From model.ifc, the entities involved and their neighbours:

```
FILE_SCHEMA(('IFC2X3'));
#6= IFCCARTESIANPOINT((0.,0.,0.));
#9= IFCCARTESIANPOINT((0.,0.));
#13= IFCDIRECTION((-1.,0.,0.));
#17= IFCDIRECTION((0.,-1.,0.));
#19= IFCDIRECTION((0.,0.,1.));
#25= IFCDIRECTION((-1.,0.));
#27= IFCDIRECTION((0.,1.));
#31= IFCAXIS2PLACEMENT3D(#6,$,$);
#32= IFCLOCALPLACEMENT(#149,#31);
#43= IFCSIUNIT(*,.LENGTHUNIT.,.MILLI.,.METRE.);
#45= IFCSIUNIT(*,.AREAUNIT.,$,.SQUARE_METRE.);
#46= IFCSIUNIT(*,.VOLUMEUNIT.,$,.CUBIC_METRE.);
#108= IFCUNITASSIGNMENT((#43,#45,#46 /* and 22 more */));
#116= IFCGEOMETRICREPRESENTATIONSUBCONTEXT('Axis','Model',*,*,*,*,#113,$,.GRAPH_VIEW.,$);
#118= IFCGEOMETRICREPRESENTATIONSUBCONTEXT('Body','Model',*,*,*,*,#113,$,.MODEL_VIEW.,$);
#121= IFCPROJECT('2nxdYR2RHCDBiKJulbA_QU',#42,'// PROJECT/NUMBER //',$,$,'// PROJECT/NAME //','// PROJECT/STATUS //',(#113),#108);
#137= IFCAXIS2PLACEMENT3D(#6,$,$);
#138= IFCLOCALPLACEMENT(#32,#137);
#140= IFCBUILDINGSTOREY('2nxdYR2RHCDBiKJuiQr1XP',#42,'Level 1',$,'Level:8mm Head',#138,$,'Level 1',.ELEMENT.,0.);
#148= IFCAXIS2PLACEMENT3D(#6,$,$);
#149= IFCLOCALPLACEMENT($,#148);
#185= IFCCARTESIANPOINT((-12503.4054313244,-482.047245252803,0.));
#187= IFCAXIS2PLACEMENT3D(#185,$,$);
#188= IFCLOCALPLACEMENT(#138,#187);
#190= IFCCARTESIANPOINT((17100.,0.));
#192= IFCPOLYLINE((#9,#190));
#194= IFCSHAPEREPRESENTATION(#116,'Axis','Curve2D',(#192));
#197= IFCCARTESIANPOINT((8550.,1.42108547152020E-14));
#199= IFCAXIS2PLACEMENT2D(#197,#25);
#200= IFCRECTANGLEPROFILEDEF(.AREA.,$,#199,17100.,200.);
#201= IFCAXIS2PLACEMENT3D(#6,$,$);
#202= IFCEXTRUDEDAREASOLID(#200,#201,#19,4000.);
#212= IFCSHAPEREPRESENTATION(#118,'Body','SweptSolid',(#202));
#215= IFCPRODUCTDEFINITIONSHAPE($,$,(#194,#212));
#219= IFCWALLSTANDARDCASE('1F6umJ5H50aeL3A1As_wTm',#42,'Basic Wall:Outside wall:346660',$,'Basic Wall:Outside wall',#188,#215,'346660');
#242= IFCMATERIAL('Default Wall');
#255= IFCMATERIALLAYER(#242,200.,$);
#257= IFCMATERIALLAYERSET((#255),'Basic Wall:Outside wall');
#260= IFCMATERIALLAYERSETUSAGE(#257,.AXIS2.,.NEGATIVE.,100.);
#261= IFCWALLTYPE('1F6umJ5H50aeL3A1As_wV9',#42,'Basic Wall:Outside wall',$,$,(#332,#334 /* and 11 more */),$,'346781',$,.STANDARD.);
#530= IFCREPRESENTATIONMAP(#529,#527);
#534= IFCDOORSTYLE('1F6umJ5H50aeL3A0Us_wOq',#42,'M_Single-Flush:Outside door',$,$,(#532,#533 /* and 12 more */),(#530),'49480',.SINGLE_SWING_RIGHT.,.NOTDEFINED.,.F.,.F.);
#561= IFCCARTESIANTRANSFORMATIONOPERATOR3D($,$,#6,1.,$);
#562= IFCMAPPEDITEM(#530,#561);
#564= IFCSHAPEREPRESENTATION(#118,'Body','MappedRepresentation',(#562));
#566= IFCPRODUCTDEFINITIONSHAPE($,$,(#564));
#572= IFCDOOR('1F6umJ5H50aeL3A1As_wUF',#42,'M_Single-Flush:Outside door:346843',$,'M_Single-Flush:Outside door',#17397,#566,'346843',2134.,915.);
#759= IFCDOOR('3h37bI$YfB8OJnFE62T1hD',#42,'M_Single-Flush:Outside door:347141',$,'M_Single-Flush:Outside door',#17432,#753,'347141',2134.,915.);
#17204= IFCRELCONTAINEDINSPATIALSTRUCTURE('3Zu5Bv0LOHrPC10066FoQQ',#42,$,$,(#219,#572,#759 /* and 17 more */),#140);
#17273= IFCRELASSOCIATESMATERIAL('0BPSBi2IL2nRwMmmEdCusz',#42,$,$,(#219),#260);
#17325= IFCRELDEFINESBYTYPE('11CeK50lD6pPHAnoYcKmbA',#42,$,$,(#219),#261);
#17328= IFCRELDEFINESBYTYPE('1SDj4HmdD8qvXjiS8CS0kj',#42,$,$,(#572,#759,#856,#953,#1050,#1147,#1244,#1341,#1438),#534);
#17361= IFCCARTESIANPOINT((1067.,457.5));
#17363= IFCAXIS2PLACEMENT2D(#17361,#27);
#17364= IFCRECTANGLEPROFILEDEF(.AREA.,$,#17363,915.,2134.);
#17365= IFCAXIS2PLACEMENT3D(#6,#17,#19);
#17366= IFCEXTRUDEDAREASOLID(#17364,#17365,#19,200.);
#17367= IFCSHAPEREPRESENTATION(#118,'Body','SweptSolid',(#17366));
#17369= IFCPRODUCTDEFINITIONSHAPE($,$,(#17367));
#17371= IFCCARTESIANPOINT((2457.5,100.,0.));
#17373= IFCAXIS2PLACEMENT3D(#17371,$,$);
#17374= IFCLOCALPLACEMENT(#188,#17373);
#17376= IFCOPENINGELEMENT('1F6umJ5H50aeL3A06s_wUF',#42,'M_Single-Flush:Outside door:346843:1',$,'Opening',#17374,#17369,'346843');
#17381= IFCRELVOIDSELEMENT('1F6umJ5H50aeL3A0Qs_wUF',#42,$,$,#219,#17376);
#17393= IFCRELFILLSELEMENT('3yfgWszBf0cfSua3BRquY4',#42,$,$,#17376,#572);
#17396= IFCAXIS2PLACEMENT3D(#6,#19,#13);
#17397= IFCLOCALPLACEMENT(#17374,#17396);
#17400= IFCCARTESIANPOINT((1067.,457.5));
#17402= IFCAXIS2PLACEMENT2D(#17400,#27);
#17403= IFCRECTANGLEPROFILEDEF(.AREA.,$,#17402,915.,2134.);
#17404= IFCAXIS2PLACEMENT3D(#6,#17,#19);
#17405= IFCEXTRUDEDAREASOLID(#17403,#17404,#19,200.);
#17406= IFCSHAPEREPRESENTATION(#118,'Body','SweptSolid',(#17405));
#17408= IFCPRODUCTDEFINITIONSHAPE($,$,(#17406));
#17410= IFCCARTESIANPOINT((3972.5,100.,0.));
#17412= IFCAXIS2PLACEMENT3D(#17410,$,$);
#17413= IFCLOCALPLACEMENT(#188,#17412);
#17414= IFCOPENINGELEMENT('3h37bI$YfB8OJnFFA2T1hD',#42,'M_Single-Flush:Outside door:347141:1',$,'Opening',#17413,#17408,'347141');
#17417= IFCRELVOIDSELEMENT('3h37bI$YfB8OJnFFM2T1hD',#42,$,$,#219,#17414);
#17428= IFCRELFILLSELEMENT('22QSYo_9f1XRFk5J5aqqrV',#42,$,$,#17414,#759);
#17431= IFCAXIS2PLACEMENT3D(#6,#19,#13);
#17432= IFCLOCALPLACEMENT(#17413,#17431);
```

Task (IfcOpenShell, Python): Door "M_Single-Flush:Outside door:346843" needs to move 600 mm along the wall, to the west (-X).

```python
import ifcopenshell
import ifcopenshell.api.geometry
import ifcopenshell.util.placement
import ifcopenshell.util.unit

model = ifcopenshell.open("model.ifc")
unit_scale = ifcopenshell.util.unit.calculate_unit_scale(model)

door = model.by_guid("1F6umJ5H50aeL3A1As_wUF")
opening = door.FillsVoids[0].RelatingOpeningElement
wall = opening.VoidsElements[0].RelatingBuildingElement

wall_matrix = ifcopenshell.util.placement.get_local_placement(wall.ObjectPlacement)
shift = wall_matrix[:3, 0] * -0.6 / unit_scale
before = ifcopenshell.util.placement.get_local_placement(door.ObjectPlacement)[:3, 3].copy()

# The door is placed relative to its opening, so it follows when the opening moves.
matrix = ifcopenshell.util.placement.get_local_placement(opening.ObjectPlacement)
matrix[:3, 3] += shift
ifcopenshell.api.geometry.edit_object_placement(
    model, product=opening, matrix=matrix, is_si=False, should_transform_children=True
)

after = ifcopenshell.util.placement.get_local_placement(door.ObjectPlacement)[:3, 3]
print("door moved by", (after - before).round(3) + 0.0)

model.write("model_edited.ifc")
```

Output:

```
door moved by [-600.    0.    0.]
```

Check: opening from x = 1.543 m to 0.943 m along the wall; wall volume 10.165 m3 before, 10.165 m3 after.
